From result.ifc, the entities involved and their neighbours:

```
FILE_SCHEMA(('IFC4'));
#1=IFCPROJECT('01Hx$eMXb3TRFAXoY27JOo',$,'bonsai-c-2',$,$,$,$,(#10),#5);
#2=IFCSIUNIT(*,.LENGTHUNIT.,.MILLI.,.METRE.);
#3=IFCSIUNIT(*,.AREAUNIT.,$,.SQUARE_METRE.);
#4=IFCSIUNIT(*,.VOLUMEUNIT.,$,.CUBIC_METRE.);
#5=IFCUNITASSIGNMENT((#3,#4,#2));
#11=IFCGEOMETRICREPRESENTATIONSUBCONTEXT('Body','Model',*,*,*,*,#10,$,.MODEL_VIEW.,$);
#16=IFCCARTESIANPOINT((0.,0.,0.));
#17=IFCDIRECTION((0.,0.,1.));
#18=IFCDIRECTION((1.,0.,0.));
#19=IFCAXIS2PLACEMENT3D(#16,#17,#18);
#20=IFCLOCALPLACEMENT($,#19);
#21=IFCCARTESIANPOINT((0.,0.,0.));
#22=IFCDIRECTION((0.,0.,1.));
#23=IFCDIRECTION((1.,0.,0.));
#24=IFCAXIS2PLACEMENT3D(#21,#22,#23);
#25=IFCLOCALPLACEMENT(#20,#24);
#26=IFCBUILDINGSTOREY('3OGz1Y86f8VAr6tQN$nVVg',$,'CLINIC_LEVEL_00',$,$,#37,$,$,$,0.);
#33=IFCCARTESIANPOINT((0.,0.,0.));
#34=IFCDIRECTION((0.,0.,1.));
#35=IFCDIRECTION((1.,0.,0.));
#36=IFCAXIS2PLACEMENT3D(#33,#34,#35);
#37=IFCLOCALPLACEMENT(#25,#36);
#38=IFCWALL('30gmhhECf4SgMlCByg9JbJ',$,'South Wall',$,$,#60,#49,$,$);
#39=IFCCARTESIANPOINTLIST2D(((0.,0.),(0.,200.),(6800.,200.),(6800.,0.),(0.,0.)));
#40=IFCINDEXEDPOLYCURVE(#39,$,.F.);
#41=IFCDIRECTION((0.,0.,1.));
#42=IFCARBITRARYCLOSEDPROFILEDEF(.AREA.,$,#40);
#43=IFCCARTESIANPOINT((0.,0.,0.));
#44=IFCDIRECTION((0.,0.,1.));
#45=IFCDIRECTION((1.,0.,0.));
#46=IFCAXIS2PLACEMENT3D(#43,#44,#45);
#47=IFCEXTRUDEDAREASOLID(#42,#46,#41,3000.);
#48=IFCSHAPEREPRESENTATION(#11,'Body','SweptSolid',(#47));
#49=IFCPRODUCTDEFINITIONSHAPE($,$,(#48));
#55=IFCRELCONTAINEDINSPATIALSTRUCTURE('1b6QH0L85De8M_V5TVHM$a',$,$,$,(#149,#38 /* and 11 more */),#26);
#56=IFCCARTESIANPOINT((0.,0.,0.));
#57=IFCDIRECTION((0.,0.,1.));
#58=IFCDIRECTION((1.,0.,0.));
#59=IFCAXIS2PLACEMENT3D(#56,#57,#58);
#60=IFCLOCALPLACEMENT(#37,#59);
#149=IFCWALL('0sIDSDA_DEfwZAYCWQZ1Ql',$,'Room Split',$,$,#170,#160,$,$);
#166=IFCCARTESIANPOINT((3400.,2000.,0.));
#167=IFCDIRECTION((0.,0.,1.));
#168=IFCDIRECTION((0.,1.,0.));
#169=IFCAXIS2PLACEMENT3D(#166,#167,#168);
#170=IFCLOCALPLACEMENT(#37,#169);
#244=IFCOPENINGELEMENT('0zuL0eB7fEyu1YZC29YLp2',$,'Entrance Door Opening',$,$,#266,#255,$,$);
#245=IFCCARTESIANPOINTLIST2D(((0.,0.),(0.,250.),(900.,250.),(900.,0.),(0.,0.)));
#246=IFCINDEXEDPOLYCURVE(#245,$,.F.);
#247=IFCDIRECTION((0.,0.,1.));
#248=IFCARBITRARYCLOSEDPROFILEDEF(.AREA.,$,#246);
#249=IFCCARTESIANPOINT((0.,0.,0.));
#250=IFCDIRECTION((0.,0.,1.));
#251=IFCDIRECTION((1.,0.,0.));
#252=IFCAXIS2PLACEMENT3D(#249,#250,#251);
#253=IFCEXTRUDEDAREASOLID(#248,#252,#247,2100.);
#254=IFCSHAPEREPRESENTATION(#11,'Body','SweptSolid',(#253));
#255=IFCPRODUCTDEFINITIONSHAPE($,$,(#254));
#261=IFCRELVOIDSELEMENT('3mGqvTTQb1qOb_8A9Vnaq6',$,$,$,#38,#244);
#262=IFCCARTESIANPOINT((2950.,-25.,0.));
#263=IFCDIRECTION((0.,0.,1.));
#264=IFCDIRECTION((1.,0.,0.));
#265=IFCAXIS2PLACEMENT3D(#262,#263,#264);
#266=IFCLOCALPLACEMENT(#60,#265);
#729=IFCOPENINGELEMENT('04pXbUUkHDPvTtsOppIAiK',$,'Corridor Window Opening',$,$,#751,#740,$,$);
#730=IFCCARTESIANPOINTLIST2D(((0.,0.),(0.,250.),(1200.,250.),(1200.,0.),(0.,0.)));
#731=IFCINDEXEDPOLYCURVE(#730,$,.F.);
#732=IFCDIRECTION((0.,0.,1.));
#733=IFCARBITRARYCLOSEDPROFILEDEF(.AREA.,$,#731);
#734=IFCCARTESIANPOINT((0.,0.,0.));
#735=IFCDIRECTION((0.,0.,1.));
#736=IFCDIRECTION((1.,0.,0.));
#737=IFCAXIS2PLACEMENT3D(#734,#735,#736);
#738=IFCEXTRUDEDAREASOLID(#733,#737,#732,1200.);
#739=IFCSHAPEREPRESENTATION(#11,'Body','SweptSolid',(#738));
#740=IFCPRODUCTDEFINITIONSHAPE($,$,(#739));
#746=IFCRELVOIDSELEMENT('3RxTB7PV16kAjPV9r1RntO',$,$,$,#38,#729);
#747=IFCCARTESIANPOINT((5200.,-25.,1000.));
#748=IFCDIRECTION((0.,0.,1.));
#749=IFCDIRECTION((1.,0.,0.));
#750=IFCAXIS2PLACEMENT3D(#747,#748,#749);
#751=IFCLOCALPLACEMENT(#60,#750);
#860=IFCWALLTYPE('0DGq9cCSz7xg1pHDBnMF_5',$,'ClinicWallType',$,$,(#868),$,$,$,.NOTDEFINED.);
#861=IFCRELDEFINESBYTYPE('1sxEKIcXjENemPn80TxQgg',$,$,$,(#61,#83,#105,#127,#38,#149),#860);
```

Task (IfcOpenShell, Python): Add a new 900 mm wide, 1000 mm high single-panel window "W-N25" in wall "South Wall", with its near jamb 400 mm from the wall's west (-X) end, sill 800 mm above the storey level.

```python
import numpy as np
import ifcopenshell
import ifcopenshell.api.feature
import ifcopenshell.api.geometry
import ifcopenshell.api.root
import ifcopenshell.api.spatial
import ifcopenshell.geom
import ifcopenshell.util.element
import ifcopenshell.util.placement
import ifcopenshell.util.representation
import ifcopenshell.util.shape
import ifcopenshell.util.unit

model = ifcopenshell.open("result.ifc")
unit_scale = ifcopenshell.util.unit.calculate_unit_scale(model)
settings = ifcopenshell.geom.settings()


def volume(element):
    """Net volume in cubic metres, openings subtracted."""
    shape = ifcopenshell.geom.create_shape(settings, element)
    return ifcopenshell.util.shape.get_volume(shape.geometry)


wall = model.by_guid("30gmhhECf4SgMlCByg9JbJ")
storey = ifcopenshell.util.element.get_container(wall, ifc_class="IfcBuildingStorey")
context = ifcopenshell.util.representation.get_context(model, "Model", "Body", "MODEL_VIEW")
before = volume(wall)

width, height, from_end, sill = 0.9, 1, 0.4, 0.8  # metres

# The wall runs along its own X axis, and the end named is its -X end.
wall_shape = ifcopenshell.geom.create_shape(settings, wall)
x, y, z = ifcopenshell.util.shape.get_vertices(wall_shape.geometry).T
start = x.min() + from_end
face, thickness = float(y.min()), float(y.max() - y.min())
wall_matrix = ifcopenshell.util.placement.get_local_placement(wall.ObjectPlacement)
level = ifcopenshell.util.placement.get_local_placement(storey.ObjectPlacement)[2, 3]


def in_wall(x, y):
    """Placement at x, y metres in the wall's axes, at sill height."""
    matrix = wall_matrix.copy()
    matrix[:, 3] = wall_matrix @ np.array([x / unit_scale, y / unit_scale, 0.0, 1.0])
    matrix[2, 3] = level + sill / unit_scale
    return matrix


# Opening: a box that overshoots both wall faces by 50 mm.
opening = ifcopenshell.api.root.create_entity(model, ifc_class="IfcOpeningElement", predefined_type="OPENING")
box = ifcopenshell.api.geometry.add_wall_representation(
    model, context=context, length=width, height=height, thickness=thickness + 0.1
)
ifcopenshell.api.geometry.assign_representation(model, product=opening, representation=box)
ifcopenshell.api.geometry.edit_object_placement(model, product=opening, matrix=in_wall(start, face - 0.05), is_si=False)
ifcopenshell.api.feature.add_feature(model, feature=opening, element=wall)

window = ifcopenshell.api.root.create_entity(model, ifc_class="IfcWindow", name="W-N25", predefined_type="WINDOW")
window.OverallWidth, window.OverallHeight = width / unit_scale, height / unit_scale
window.PartitioningType = "SINGLE_PANEL"
body = ifcopenshell.api.geometry.add_window_representation(
    model,
    context=context,
    overall_width=window.OverallWidth,
    overall_height=window.OverallHeight,
    partition_type="SINGLE_PANEL",
)
ifcopenshell.api.geometry.assign_representation(model, product=window, representation=body)
ifcopenshell.api.spatial.assign_container(model, products=[window], relating_structure=storey)
ifcopenshell.api.feature.add_filling(model, opening=opening, element=window)

# Centre the window in the wall's thickness.
ifcopenshell.api.geometry.edit_object_placement(model, product=window, matrix=in_wall(start, face), is_si=False)
window_shape = ifcopenshell.geom.create_shape(settings, window)
depth = ifcopenshell.util.shape.get_vertices(window_shape.geometry)[:, 1]
offset = face + thickness / 2 - (depth.min() + depth.max()) / 2
ifcopenshell.api.geometry.edit_object_placement(model, product=window, matrix=in_wall(start, offset), is_si=False)

after = volume(wall)

print(f"wall volume {before:.3f} -> {after:.3f} m3")

model.write("result_v2.ifc")
```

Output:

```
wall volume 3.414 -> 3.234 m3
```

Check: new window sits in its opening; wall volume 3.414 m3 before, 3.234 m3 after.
